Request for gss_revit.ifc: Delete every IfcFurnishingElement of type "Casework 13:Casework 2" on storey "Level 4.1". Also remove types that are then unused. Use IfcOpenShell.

First a look at what the model holds.

```python
import ifcopenshell
import ifcopenshell.util.element

model = ifcopenshell.open("gss_revit.ifc")
print(model.schema)
storey = next(s for s in model.by_type("IfcBuildingStorey") if s.Name == "Level 4.1")
furniture = [e for e in ifcopenshell.util.element.get_decomposition(storey) if e.is_a("IfcFurnishingElement")]
seen = {}
for e in furniture:
    element_type = ifcopenshell.util.element.get_type(e)
    name = element_type.Name if element_type not in (None, e) else None
    seen[name] = seen.get(name, 0) + 1
for name, count in sorted(seen.items(), key=str):
    print(count, "x", name)
```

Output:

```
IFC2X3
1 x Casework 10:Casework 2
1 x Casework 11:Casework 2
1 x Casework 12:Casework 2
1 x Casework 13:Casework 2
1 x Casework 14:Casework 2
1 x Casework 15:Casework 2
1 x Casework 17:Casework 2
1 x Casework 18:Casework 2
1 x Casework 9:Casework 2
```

```python
import ifcopenshell
import ifcopenshell.api.root
import ifcopenshell.util.element

model = ifcopenshell.open("gss_revit.ifc")

storey = next(s for s in model.by_type("IfcBuildingStorey") if s.Name == "Level 4.1")
furniture = [e for e in ifcopenshell.util.element.get_decomposition(storey) if e.is_a("IfcFurnishingElement")]
targets = [e for e in furniture if (t := ifcopenshell.util.element.get_type(e)) not in (None, e) and t.Name == "Casework 13:Casework 2"]
types = {ifcopenshell.util.element.get_type(e) for e in targets} - {None, *targets}

for e in targets:
    ifcopenshell.api.root.remove_product(model, product=e)
print(len(targets), "removed")

unused = [t for t in types if not ifcopenshell.util.element.get_types(t)]
for t in unused:
    ifcopenshell.api.root.remove_product(model, product=t)
print(len(unused), "unused types removed")

model.write("gss_revit_edited.ifc")
```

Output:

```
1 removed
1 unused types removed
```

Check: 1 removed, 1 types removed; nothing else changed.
